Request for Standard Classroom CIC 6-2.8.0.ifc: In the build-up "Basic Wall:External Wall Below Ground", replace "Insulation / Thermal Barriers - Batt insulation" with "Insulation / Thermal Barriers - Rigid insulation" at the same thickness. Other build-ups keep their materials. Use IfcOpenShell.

First a look at what the model holds.

```python
import ifcopenshell
import ifcopenshell.util.element

model = ifcopenshell.open("Standard Classroom CIC 6-2.8.0.ifc")
print(model.schema)
for layer_set in model.by_type("IfcMaterialLayerSet"):
    if layer_set.LayerSetName == "Basic Wall:External Wall Below Ground":
        for layer in layer_set.MaterialLayers:
            print(layer.id(), layer.Material and layer.Material.Name, layer.LayerThickness, sep=" | ")
        print(len(ifcopenshell.util.element.get_elements_by_material(model, layer_set)), "elements and types use it")
print(sorted(m.Name for m in model.by_type("IfcMaterial") if m.Name)[:60])
```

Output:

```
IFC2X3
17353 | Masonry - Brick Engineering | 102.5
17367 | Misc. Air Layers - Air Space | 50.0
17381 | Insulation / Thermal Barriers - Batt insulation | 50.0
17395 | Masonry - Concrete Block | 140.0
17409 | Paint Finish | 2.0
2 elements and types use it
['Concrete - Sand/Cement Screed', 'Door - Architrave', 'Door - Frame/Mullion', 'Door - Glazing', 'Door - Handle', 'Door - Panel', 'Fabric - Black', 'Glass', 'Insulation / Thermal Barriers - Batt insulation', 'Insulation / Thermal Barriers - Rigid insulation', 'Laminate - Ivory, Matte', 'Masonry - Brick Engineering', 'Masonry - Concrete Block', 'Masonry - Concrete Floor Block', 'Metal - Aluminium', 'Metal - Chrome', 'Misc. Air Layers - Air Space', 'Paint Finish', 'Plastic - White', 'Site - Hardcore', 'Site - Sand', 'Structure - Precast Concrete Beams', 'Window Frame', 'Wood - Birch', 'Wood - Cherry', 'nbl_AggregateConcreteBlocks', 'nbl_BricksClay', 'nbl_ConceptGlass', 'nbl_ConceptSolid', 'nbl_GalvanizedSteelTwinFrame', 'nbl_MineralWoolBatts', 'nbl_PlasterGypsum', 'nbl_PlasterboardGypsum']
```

```python
import ifcopenshell
import ifcopenshell.api.material

model = ifcopenshell.open("Standard Classroom CIC 6-2.8.0.ifc")

layer_set = next(s for s in model.by_type("IfcMaterialLayerSet") if s.LayerSetName == "Basic Wall:External Wall Below Ground")
layer = next(l for l in layer_set.MaterialLayers if l.Material and l.Material.Name == "Insulation / Thermal Barriers - Batt insulation")
material = next(m for m in model.by_type("IfcMaterial") if m.Name == "Insulation / Thermal Barriers - Rigid insulation")

# Point this one layer at the other material; renaming the old one would change it everywhere.
ifcopenshell.api.material.edit_layer(model, layer=layer, attributes={}, material=material)

print([l.Material.Name if l.Material else None for l in layer_set.MaterialLayers])

model.write("Standard Classroom CIC 6-2.8.0_v2.ifc")
```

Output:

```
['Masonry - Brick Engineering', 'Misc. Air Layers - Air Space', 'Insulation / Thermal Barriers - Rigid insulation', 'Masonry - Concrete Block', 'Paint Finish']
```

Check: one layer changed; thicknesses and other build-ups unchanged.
